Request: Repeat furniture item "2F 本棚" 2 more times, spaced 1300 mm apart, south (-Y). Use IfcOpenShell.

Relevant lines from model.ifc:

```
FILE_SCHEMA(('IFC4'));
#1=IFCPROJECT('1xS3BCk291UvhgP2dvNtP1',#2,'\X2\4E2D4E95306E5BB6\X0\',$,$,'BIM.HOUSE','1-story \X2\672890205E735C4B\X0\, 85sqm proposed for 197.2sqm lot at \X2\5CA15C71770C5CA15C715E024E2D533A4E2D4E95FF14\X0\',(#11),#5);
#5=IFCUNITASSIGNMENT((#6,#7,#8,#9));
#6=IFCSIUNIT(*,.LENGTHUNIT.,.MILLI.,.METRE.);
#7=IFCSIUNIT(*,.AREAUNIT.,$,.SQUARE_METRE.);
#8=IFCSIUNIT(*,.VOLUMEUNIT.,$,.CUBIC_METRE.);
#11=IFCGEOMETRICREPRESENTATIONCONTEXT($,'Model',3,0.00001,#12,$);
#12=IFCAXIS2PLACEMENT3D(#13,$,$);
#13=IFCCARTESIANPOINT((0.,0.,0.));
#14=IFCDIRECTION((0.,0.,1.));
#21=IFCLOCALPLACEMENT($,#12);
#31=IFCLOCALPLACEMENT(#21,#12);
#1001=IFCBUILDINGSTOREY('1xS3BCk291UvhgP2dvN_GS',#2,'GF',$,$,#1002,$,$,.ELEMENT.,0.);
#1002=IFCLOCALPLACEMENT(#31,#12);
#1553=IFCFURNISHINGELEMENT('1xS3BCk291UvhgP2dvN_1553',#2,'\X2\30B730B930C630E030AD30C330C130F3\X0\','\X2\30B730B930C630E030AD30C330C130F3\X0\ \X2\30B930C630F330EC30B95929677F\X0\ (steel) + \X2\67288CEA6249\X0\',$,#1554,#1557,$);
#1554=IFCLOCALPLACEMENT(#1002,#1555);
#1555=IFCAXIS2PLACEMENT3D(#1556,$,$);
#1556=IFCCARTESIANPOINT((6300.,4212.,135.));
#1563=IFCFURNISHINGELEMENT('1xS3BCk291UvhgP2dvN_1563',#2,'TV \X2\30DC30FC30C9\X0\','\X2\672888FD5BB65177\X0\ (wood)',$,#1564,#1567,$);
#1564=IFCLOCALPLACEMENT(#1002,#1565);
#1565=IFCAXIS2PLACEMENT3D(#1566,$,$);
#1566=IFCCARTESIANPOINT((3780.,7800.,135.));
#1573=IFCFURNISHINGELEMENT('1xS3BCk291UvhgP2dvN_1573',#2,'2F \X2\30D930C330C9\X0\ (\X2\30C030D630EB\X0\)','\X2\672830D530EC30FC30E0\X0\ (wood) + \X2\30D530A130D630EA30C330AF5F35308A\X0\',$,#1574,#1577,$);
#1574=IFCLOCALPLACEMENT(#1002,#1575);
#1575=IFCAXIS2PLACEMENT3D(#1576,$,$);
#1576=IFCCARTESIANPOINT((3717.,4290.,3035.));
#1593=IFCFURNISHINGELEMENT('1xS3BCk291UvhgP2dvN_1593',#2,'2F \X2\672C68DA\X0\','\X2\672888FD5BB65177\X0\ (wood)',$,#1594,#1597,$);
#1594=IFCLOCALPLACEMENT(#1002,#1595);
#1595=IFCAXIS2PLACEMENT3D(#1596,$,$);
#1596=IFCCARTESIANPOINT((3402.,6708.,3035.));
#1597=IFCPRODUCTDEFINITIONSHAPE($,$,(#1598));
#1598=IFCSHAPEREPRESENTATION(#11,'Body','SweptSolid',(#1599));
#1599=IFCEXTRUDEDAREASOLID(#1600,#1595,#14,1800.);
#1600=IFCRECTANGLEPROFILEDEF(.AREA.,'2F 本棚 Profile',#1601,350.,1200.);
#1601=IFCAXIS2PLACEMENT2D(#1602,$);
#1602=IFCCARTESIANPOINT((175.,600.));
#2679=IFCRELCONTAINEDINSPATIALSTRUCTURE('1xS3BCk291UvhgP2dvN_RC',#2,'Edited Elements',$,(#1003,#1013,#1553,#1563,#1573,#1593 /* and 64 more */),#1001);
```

```python
import numpy as np
import ifcopenshell
import ifcopenshell.api.geometry
import ifcopenshell.api.root
import ifcopenshell.util.element
import ifcopenshell.util.placement
import ifcopenshell.util.unit

model = ifcopenshell.open("model.ifc")
unit_scale = ifcopenshell.util.unit.calculate_unit_scale(model)


def reuse_history(source, copy):
    """copy_class also copies each property set's owner history, people and application; keep the originals."""
    for rel in copy.IsDefinedBy:
        if rel.is_a("IfcRelDefinesByProperties") and (history := rel.RelatingPropertyDefinition.OwnerHistory):
            rel.RelatingPropertyDefinition.OwnerHistory = source.OwnerHistory
            ifcopenshell.util.element.remove_deep2(model, history)


source = model.by_guid("1xS3BCk291UvhgP2dvN_1593")
base = ifcopenshell.util.placement.get_local_placement(source.ObjectPlacement)
step = np.array([0.0, -1.0, 0.0]) * 1.3 / unit_scale

for i in range(1, 3):
    copy = ifcopenshell.api.root.copy_class(model, product=source)
    copy.Representation = ifcopenshell.util.element.copy_deep(
        model, source.Representation, exclude=["IfcGeometricRepresentationContext", "IfcRepresentationMap"]
    )
    reuse_history(source, copy)
    matrix = base.copy()
    matrix[:3, 3] += i * step
    print("added at", matrix[:3, 3].round(3) + 0.0)
    ifcopenshell.api.geometry.edit_object_placement(model, product=copy, matrix=matrix, is_si=False)

model.write("model_updated.ifc")
```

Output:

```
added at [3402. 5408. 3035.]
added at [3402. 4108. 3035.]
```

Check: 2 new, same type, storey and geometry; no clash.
